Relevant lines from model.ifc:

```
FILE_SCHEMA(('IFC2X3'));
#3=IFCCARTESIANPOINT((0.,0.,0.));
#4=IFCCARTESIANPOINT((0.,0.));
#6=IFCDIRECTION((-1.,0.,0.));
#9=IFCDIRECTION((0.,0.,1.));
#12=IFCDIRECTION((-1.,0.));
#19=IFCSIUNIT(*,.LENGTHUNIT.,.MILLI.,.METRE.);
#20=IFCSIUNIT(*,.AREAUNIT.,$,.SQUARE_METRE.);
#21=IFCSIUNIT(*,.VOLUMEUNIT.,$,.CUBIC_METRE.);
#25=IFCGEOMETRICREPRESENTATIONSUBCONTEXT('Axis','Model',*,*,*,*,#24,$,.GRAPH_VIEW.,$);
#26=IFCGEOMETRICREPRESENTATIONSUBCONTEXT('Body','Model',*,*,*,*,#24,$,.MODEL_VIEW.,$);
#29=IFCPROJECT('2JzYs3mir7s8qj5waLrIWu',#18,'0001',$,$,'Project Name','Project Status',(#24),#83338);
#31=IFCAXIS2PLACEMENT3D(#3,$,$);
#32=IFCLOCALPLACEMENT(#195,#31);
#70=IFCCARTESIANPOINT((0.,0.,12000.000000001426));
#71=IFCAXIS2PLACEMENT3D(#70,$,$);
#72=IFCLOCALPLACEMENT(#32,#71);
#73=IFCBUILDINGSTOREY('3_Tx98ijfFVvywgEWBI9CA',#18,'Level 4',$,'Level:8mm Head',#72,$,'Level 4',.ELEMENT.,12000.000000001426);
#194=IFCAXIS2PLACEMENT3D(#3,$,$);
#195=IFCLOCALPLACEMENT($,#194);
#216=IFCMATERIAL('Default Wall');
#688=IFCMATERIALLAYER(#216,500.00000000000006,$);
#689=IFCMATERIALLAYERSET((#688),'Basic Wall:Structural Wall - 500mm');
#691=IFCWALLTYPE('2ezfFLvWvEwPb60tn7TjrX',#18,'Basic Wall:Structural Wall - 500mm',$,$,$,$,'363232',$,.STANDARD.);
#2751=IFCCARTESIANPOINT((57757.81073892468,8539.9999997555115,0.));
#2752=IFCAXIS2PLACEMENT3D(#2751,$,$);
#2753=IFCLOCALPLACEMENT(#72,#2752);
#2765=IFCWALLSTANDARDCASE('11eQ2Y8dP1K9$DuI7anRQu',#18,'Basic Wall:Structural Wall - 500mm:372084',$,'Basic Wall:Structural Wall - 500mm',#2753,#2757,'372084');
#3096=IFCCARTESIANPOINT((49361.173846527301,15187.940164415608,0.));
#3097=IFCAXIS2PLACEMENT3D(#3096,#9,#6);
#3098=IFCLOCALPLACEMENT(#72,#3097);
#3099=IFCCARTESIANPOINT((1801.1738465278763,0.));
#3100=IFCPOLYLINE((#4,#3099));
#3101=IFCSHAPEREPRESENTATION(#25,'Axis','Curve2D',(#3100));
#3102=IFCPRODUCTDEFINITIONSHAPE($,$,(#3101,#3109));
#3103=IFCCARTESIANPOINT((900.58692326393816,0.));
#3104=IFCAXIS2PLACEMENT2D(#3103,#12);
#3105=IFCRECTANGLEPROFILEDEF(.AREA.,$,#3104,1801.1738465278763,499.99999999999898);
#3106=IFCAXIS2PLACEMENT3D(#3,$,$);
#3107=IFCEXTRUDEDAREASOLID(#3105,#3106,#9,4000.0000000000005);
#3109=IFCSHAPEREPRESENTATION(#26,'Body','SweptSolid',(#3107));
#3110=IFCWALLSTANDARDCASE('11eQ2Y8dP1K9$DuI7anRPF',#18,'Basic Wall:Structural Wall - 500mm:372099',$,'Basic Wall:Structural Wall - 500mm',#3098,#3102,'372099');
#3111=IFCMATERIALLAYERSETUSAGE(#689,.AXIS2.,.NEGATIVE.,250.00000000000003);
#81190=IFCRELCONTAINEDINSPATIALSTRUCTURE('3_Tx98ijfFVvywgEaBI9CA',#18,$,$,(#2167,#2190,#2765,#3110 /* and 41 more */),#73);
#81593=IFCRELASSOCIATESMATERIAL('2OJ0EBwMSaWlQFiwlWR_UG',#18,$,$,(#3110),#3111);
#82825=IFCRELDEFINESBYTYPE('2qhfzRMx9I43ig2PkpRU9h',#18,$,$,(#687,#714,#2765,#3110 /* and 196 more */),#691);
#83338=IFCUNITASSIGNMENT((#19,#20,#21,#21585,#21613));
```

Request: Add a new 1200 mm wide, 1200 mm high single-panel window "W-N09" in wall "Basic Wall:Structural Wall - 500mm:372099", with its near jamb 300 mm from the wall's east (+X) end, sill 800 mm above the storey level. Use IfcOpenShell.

```python
import numpy as np
import ifcopenshell
import ifcopenshell.api.feature
import ifcopenshell.api.geometry
import ifcopenshell.api.root
import ifcopenshell.api.spatial
import ifcopenshell.api.type
import ifcopenshell.geom
import ifcopenshell.util.element
import ifcopenshell.util.placement
import ifcopenshell.util.representation
import ifcopenshell.util.shape
import ifcopenshell.util.unit

model = ifcopenshell.open("model.ifc")
unit_scale = ifcopenshell.util.unit.calculate_unit_scale(model)
settings = ifcopenshell.geom.settings()


def volume(element):
    """Net volume in cubic metres, openings subtracted."""
    shape = ifcopenshell.geom.create_shape(settings, element)
    return ifcopenshell.util.shape.get_volume(shape.geometry)


wall = model.by_guid("11eQ2Y8dP1K9$DuI7anRPF")
storey = ifcopenshell.util.element.get_container(wall, ifc_class="IfcBuildingStorey")
context = ifcopenshell.util.representation.get_context(model, "Model", "Body", "MODEL_VIEW")
before = volume(wall)

width, height, from_end, sill = 1.2, 1.2, 0.3, 0.8  # metres

# The wall runs along its own X axis, and the end named is its -X end.
wall_shape = ifcopenshell.geom.create_shape(settings, wall)
x, y, z = ifcopenshell.util.shape.get_vertices(wall_shape.geometry).T
start = x.min() + from_end
face, thickness = float(y.min()), float(y.max() - y.min())
wall_matrix = ifcopenshell.util.placement.get_local_placement(wall.ObjectPlacement)
level = ifcopenshell.util.placement.get_local_placement(storey.ObjectPlacement)[2, 3]


def in_wall(x, y):
    """Placement at x, y metres in the wall's axes, at sill height."""
    matrix = wall_matrix.copy()
    matrix[:, 3] = wall_matrix @ np.array([x / unit_scale, y / unit_scale, 0.0, 1.0])
    matrix[2, 3] = level + sill / unit_scale
    return matrix


# Opening: a box that overshoots both wall faces by 50 mm.
opening = ifcopenshell.api.root.create_entity(model, ifc_class="IfcOpeningElement")
box = ifcopenshell.api.geometry.add_wall_representation(
    model, context=context, length=width, height=height, thickness=thickness + 0.1
)
ifcopenshell.api.geometry.assign_representation(model, product=opening, representation=box)
ifcopenshell.api.geometry.edit_object_placement(model, product=opening, matrix=in_wall(start, face - 0.05), is_si=False)
ifcopenshell.api.feature.add_feature(model, feature=opening, element=wall)

window = ifcopenshell.api.root.create_entity(model, ifc_class="IfcWindow", name="W-N09")
window.OverallWidth, window.OverallHeight = width / unit_scale, height / unit_scale
body = ifcopenshell.api.geometry.add_window_representation(
    model,
    context=context,
    overall_width=window.OverallWidth,
    overall_height=window.OverallHeight,
    partition_type="SINGLE_PANEL",
)
ifcopenshell.api.geometry.assign_representation(model, product=window, representation=body)
ifcopenshell.api.spatial.assign_container(model, products=[window], relating_structure=storey)
fills = ifcopenshell.api.feature.add_filling(model, opening=opening, element=window)
fills.OwnerHistory = window.OwnerHistory  # required in IFC2X3

# IFC2X3 keeps the operation on the window style.
style = ifcopenshell.api.root.create_entity(model, ifc_class="IfcWindowStyle", name="W-N09")
style.OperationType, style.ConstructionType = "SINGLE_PANEL", "NOTDEFINED"
style.ParameterTakesPrecedence = style.Sizeable = False
ifcopenshell.api.type.assign_type(model, related_objects=[window], relating_type=style)

# Centre the window in the wall's thickness.
ifcopenshell.api.geometry.edit_object_placement(model, product=window, matrix=in_wall(start, face), is_si=False)
window_shape = ifcopenshell.geom.create_shape(settings, window)
depth = ifcopenshell.util.shape.get_vertices(window_shape.geometry)[:, 1]
offset = face + thickness / 2 - (depth.min() + depth.max()) / 2
ifcopenshell.api.geometry.edit_object_placement(model, product=window, matrix=in_wall(start, offset), is_si=False)

after = volume(wall)

print(f"wall volume {before:.3f} -> {after:.3f} m3")

model.write("model_edited.ifc")
```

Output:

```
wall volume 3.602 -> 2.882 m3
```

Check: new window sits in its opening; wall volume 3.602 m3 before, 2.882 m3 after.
